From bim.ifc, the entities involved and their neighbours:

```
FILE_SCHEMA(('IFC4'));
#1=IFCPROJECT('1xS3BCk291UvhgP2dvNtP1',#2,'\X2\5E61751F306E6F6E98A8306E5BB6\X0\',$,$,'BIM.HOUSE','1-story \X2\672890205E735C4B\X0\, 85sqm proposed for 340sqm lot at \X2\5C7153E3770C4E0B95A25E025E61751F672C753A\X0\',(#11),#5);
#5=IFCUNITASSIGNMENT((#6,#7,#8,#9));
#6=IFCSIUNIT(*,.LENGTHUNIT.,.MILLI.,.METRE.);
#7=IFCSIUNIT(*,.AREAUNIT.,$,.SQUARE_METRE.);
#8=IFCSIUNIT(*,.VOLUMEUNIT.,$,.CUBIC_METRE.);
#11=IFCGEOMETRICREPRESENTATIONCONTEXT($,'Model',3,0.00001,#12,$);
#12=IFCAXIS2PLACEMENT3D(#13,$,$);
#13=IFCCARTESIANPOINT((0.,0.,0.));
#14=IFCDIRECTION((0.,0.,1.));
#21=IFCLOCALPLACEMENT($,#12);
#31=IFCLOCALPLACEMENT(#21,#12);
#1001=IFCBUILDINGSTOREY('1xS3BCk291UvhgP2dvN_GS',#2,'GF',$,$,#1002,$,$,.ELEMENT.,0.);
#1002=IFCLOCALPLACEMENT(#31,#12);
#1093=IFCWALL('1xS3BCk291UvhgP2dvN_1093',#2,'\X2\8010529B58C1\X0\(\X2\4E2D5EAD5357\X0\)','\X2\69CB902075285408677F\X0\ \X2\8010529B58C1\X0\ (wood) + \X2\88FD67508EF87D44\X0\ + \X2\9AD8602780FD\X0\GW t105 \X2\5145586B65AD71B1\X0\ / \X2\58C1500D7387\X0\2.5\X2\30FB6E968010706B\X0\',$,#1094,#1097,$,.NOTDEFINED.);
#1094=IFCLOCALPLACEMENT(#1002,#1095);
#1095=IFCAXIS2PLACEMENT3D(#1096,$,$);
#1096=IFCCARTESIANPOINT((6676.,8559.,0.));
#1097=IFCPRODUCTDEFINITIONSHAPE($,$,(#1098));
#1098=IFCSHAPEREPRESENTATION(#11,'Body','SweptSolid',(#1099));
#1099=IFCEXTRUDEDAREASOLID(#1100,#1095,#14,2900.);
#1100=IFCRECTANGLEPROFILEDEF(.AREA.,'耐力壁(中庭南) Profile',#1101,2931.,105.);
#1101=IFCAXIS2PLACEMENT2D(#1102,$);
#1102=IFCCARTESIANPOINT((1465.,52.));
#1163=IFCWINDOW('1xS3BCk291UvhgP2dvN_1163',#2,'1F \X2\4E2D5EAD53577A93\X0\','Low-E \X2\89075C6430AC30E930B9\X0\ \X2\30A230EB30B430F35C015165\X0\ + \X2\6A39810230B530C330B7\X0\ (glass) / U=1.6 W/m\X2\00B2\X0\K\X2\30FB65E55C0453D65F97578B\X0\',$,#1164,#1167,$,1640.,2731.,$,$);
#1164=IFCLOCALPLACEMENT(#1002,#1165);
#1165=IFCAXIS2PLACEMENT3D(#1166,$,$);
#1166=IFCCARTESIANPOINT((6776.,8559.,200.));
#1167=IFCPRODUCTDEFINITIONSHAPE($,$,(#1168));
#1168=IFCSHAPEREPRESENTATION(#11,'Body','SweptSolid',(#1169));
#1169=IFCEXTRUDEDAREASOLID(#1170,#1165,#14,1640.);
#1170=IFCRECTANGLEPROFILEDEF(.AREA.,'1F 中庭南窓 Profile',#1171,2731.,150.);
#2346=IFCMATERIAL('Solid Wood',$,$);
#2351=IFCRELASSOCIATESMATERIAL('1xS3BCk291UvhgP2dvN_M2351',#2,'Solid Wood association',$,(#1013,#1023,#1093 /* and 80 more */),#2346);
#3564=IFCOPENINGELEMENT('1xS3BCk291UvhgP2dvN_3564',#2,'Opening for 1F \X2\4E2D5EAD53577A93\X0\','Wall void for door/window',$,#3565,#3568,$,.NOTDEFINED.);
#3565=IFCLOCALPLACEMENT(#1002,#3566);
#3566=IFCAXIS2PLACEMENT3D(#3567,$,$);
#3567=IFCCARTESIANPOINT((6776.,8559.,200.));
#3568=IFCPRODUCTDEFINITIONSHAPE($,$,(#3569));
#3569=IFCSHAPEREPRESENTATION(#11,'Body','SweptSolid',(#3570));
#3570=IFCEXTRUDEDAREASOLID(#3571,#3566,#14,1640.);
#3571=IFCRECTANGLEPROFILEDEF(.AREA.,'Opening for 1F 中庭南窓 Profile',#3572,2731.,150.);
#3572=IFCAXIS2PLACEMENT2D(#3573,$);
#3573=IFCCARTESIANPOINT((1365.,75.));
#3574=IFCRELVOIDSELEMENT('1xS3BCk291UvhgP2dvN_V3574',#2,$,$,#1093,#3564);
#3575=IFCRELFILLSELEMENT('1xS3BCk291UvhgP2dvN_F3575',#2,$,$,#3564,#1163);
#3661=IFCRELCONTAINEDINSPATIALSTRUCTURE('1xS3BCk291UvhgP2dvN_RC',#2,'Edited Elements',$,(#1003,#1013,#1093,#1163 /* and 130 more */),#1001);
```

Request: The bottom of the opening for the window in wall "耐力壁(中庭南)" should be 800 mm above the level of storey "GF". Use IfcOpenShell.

```python
import numpy as np
import ifcopenshell
import ifcopenshell.api.geometry
import ifcopenshell.geom
import ifcopenshell.util.element
import ifcopenshell.util.placement
import ifcopenshell.util.shape
import ifcopenshell.util.unit

model = ifcopenshell.open("bim.ifc")
unit_scale = ifcopenshell.util.unit.calculate_unit_scale(model)

window = model.by_guid("1xS3BCk291UvhgP2dvN_1163")
opening = window.FillsVoids[0].RelatingOpeningElement
storey = ifcopenshell.util.element.get_container(window, ifc_class="IfcBuildingStorey")
level = ifcopenshell.util.placement.get_local_placement(storey.ObjectPlacement)[2, 3]

# The opening's origin need not be at the sill, so measure its lowest point.
shape = ifcopenshell.geom.create_shape(ifcopenshell.geom.settings(), opening)
bottom = ifcopenshell.util.shape.get_shape_bottom_elevation(shape, shape.geometry) / unit_scale
dz = level + 0.8 / unit_scale - bottom

shift = np.array([0.0, 0.0, dz])
# The window is not placed relative to its opening, so move both.
for product in (opening, window):
    matrix = ifcopenshell.util.placement.get_local_placement(product.ObjectPlacement)
    matrix[:3, 3] += shift
    ifcopenshell.api.geometry.edit_object_placement(model, product=product, matrix=matrix, is_si=False)

print(f"moved by {dz * unit_scale:+.3f} m")

model.write("bim_v2.ifc")
```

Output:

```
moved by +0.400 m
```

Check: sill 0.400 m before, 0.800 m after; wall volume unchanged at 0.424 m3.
